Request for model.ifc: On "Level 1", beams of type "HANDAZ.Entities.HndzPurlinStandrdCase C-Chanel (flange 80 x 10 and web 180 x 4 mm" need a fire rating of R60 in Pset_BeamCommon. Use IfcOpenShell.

First a look at what the model holds.

```python
import ifcopenshell
import ifcopenshell.util.element

model = ifcopenshell.open("model.ifc")
print(model.schema)
storey = next(s for s in model.by_type("IfcBuildingStorey") if s.Name == "Level 1")
beams = [e for e in ifcopenshell.util.element.get_decomposition(storey) if e.is_a("IfcBeam")]
seen = {}
for e in beams:
    element_type = ifcopenshell.util.element.get_type(e)
    key = (element_type.Name if element_type != e and element_type else None, ifcopenshell.util.element.get_pset(e, "Pset_BeamCommon", "FireRating"))
    seen[key] = seen.get(key, 0) + 1
for (name, value), count in sorted(seen.items(), key=str):
    print(count, "x", name, "|", value)
```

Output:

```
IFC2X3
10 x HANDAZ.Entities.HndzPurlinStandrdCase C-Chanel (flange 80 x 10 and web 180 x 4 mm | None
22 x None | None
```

```python
import ifcopenshell
import ifcopenshell.api.pset
import ifcopenshell.util.element

model = ifcopenshell.open("model.ifc")

storey = next(s for s in model.by_type("IfcBuildingStorey") if s.Name == "Level 1")
beams = [e for e in ifcopenshell.util.element.get_decomposition(storey) if e.is_a("IfcBeam")]

count = 0
for e in beams:
    element_type = ifcopenshell.util.element.get_type(e)
    if element_type in (None, e) or element_type.Name != "HANDAZ.Entities.HndzPurlinStandrdCase C-Chanel (flange 80 x 10 and web 180 x 4 mm":
        continue
    # add_pset returns the element's existing set when there is one.
    pset = ifcopenshell.api.pset.add_pset(model, product=e, name="Pset_BeamCommon")
    ifcopenshell.api.pset.edit_pset(model, pset=pset, properties={"FireRating": "R60"})
    count += 1

print(count, "beams updated")

model.write("model_edited.ifc")
```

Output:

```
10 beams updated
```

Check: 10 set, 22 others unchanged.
